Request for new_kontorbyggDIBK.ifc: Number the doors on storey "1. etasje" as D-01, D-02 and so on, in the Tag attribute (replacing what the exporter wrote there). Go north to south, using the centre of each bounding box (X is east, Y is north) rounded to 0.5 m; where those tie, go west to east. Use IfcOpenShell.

First a look at what the model holds.

```python
import ifcopenshell
import ifcopenshell.util.element
import ifcopenshell.util.placement

model = ifcopenshell.open("new_kontorbyggDIBK.ifc")
print(model.schema)
storey = next(s for s in model.by_type("IfcBuildingStorey") if s.Name == "1. etasje")
doors = [e for e in ifcopenshell.util.element.get_decomposition(storey) if e.is_a("IfcDoor")]
for e in sorted(doors, key=lambda e: e.id()):
    origin = ifcopenshell.util.placement.get_local_placement(e.ObjectPlacement)[:3, 3]
    print(e.id(), e.Tag, e.Name, origin.round(2) + 0.0, sep=" | ")
```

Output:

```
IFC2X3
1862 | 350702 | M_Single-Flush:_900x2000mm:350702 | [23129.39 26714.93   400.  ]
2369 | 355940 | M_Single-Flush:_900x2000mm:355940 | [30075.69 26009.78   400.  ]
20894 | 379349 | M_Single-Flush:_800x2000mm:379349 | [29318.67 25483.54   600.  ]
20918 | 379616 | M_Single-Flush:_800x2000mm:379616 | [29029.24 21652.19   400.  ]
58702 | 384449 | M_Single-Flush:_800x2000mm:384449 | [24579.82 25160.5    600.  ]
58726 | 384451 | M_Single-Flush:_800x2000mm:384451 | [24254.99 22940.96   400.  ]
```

```python
import ifcopenshell
import ifcopenshell.geom
import ifcopenshell.util.element
import ifcopenshell.util.shape

model = ifcopenshell.open("new_kontorbyggDIBK.ifc")
settings = ifcopenshell.geom.settings()
settings.set("use-world-coords", True)


def centre(element):
    shape = ifcopenshell.geom.create_shape(settings, element)
    return ifcopenshell.util.shape.get_bbox_centroid(shape.geometry)


storey = next(s for s in model.by_type("IfcBuildingStorey") if s.Name == "1. etasje")
doors = [e for e in ifcopenshell.util.element.get_decomposition(storey) if e.is_a("IfcDoor")]

# Insertion points can sit at a corner or the storey origin, so sort by the geometry (in metres).
centres = {e: centre(e) for e in doors}
doors.sort(key=lambda e: (-round(centres[e][1] / 0.5), centres[e][0]))

for i, e in enumerate(doors, start=1):
    number = f"D-{i:02d}"
    e.Tag = number
    print(e.id(), number)

model.write("new_kontorbyggDIBK_rev.ifc")
```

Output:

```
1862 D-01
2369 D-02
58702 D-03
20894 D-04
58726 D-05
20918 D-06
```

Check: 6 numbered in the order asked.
